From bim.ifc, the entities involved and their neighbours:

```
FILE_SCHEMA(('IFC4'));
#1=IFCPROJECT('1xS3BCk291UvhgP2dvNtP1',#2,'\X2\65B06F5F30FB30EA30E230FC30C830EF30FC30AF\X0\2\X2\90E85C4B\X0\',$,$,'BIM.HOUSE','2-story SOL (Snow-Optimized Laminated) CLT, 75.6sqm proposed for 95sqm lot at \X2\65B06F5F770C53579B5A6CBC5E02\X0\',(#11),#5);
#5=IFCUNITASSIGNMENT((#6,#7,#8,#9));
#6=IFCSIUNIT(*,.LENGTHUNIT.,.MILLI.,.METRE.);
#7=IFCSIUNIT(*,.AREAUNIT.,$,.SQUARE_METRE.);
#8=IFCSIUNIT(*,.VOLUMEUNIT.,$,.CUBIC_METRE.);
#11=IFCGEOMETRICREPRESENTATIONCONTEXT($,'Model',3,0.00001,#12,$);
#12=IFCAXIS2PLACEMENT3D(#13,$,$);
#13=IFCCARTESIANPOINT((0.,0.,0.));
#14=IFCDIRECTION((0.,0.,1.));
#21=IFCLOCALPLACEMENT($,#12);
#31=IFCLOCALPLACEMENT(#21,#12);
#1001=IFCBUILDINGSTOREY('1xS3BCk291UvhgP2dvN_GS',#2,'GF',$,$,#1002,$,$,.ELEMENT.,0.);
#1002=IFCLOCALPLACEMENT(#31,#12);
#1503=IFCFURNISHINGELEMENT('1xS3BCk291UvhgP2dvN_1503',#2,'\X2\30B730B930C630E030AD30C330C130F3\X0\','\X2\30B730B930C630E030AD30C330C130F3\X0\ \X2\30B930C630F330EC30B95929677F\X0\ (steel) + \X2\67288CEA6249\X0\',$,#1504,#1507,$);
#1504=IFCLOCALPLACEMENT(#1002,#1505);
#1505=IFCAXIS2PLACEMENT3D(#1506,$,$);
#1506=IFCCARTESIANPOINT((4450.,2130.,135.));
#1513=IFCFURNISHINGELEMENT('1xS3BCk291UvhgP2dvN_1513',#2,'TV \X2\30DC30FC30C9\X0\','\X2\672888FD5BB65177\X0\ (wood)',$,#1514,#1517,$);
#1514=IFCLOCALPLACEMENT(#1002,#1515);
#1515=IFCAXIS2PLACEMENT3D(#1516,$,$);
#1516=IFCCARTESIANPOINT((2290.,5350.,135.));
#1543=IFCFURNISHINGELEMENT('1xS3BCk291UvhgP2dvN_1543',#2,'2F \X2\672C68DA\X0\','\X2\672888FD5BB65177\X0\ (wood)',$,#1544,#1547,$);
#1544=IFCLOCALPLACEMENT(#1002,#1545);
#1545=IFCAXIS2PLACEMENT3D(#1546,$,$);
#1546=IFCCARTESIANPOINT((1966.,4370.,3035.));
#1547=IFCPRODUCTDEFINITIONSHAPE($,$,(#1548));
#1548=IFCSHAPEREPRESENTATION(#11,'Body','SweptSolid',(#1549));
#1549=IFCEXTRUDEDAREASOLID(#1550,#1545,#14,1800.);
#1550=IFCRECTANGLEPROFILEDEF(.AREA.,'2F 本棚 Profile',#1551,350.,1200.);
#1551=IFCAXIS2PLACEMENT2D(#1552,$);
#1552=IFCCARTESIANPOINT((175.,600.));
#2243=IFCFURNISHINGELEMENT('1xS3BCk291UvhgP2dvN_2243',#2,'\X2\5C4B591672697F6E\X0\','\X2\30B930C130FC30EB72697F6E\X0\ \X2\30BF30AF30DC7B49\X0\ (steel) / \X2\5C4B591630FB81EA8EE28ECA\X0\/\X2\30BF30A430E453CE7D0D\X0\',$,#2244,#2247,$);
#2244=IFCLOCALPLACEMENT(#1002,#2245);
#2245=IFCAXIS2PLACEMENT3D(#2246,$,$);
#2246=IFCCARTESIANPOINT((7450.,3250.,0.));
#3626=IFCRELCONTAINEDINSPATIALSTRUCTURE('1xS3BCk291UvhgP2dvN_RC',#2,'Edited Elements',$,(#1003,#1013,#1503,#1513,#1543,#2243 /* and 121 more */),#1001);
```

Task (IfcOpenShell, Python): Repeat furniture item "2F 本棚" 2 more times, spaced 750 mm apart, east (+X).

```python
import numpy as np
import ifcopenshell
import ifcopenshell.api.geometry
import ifcopenshell.api.root
import ifcopenshell.util.element
import ifcopenshell.util.placement
import ifcopenshell.util.unit

model = ifcopenshell.open("bim.ifc")
unit_scale = ifcopenshell.util.unit.calculate_unit_scale(model)


def reuse_history(source, copy):
    """copy_class also copies each property set's owner history, people and application; keep the originals."""
    for rel in copy.IsDefinedBy:
        if rel.is_a("IfcRelDefinesByProperties") and (history := rel.RelatingPropertyDefinition.OwnerHistory):
            rel.RelatingPropertyDefinition.OwnerHistory = source.OwnerHistory
            ifcopenshell.util.element.remove_deep2(model, history)


source = model.by_guid("1xS3BCk291UvhgP2dvN_1543")
base = ifcopenshell.util.placement.get_local_placement(source.ObjectPlacement)
step = np.array([1.0, 0.0, 0.0]) * 0.75 / unit_scale

for i in range(1, 3):
    copy = ifcopenshell.api.root.copy_class(model, product=source)
    copy.Representation = ifcopenshell.util.element.copy_deep(
        model, source.Representation, exclude=["IfcGeometricRepresentationContext", "IfcRepresentationMap"]
    )
    reuse_history(source, copy)
    matrix = base.copy()
    matrix[:3, 3] += i * step
    print("added at", matrix[:3, 3].round(3) + 0.0)
    ifcopenshell.api.geometry.edit_object_placement(model, product=copy, matrix=matrix, is_si=False)

model.write("bim_edited.ifc")
```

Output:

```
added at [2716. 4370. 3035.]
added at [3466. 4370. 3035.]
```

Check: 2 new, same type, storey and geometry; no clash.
